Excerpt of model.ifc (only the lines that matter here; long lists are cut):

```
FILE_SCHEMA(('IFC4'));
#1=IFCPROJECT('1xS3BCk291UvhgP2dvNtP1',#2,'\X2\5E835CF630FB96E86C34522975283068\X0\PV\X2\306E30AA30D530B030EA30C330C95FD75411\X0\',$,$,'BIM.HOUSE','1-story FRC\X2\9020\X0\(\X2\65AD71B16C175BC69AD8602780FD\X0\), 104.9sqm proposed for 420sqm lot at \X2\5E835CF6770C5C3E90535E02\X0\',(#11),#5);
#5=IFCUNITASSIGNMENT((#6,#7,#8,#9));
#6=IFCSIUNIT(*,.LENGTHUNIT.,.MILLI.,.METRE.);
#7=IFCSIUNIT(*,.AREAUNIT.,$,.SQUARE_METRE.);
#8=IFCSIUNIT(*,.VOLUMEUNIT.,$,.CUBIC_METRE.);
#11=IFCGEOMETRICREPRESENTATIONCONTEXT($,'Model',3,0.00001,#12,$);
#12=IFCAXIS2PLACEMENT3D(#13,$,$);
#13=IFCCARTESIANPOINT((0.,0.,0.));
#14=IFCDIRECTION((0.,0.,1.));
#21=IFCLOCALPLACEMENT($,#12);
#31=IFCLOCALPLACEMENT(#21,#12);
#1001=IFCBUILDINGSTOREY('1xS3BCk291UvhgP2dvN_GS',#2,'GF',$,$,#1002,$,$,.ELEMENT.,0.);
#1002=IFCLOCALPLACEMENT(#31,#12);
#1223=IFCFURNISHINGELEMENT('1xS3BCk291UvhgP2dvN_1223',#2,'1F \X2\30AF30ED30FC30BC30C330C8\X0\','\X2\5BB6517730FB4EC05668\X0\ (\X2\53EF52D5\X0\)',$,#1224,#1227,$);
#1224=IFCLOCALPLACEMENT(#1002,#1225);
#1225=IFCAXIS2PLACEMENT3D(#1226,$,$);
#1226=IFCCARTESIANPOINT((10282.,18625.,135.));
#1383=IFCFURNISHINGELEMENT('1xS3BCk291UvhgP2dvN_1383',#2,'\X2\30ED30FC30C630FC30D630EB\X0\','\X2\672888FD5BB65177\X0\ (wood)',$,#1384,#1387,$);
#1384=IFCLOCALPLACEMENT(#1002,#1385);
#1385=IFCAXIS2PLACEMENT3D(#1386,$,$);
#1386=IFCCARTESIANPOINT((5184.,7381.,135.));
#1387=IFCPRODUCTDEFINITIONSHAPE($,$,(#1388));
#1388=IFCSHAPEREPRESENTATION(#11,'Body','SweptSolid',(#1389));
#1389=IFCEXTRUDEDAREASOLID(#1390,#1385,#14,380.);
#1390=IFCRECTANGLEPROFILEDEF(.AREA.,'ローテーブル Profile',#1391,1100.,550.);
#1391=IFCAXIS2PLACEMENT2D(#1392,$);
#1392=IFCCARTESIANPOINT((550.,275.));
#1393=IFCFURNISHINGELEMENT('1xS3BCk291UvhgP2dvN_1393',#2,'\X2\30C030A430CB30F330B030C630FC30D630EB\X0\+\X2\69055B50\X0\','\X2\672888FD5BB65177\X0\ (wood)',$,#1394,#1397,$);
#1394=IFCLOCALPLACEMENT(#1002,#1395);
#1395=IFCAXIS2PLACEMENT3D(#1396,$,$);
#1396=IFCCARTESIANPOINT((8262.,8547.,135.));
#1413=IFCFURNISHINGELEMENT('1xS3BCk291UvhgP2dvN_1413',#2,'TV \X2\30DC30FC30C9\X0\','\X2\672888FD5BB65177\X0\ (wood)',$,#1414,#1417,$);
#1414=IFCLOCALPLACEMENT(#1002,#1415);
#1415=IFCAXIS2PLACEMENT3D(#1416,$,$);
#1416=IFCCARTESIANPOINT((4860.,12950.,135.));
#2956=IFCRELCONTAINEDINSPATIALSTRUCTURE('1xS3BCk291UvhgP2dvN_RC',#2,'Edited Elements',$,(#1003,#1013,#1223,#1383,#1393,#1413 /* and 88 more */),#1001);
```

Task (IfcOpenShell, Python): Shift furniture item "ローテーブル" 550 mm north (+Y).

```python
import ifcopenshell
import ifcopenshell.api.geometry
import ifcopenshell.util.placement
import ifcopenshell.util.unit

model = ifcopenshell.open("model.ifc")
unit_scale = ifcopenshell.util.unit.calculate_unit_scale(model)

item = model.by_guid("1xS3BCk291UvhgP2dvN_1383")
matrix = ifcopenshell.util.placement.get_local_placement(item.ObjectPlacement)
matrix[1, 3] += 0.55 / unit_scale
ifcopenshell.api.geometry.edit_object_placement(model, product=item, matrix=matrix, is_si=False)

print(ifcopenshell.util.placement.get_local_placement(item.ObjectPlacement).round(3) + 0.0)

model.write("model_rev.ifc")
```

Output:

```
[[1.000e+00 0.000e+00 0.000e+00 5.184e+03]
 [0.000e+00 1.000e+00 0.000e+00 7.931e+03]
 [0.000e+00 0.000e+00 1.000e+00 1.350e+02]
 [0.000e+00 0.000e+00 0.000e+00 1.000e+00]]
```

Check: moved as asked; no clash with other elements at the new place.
